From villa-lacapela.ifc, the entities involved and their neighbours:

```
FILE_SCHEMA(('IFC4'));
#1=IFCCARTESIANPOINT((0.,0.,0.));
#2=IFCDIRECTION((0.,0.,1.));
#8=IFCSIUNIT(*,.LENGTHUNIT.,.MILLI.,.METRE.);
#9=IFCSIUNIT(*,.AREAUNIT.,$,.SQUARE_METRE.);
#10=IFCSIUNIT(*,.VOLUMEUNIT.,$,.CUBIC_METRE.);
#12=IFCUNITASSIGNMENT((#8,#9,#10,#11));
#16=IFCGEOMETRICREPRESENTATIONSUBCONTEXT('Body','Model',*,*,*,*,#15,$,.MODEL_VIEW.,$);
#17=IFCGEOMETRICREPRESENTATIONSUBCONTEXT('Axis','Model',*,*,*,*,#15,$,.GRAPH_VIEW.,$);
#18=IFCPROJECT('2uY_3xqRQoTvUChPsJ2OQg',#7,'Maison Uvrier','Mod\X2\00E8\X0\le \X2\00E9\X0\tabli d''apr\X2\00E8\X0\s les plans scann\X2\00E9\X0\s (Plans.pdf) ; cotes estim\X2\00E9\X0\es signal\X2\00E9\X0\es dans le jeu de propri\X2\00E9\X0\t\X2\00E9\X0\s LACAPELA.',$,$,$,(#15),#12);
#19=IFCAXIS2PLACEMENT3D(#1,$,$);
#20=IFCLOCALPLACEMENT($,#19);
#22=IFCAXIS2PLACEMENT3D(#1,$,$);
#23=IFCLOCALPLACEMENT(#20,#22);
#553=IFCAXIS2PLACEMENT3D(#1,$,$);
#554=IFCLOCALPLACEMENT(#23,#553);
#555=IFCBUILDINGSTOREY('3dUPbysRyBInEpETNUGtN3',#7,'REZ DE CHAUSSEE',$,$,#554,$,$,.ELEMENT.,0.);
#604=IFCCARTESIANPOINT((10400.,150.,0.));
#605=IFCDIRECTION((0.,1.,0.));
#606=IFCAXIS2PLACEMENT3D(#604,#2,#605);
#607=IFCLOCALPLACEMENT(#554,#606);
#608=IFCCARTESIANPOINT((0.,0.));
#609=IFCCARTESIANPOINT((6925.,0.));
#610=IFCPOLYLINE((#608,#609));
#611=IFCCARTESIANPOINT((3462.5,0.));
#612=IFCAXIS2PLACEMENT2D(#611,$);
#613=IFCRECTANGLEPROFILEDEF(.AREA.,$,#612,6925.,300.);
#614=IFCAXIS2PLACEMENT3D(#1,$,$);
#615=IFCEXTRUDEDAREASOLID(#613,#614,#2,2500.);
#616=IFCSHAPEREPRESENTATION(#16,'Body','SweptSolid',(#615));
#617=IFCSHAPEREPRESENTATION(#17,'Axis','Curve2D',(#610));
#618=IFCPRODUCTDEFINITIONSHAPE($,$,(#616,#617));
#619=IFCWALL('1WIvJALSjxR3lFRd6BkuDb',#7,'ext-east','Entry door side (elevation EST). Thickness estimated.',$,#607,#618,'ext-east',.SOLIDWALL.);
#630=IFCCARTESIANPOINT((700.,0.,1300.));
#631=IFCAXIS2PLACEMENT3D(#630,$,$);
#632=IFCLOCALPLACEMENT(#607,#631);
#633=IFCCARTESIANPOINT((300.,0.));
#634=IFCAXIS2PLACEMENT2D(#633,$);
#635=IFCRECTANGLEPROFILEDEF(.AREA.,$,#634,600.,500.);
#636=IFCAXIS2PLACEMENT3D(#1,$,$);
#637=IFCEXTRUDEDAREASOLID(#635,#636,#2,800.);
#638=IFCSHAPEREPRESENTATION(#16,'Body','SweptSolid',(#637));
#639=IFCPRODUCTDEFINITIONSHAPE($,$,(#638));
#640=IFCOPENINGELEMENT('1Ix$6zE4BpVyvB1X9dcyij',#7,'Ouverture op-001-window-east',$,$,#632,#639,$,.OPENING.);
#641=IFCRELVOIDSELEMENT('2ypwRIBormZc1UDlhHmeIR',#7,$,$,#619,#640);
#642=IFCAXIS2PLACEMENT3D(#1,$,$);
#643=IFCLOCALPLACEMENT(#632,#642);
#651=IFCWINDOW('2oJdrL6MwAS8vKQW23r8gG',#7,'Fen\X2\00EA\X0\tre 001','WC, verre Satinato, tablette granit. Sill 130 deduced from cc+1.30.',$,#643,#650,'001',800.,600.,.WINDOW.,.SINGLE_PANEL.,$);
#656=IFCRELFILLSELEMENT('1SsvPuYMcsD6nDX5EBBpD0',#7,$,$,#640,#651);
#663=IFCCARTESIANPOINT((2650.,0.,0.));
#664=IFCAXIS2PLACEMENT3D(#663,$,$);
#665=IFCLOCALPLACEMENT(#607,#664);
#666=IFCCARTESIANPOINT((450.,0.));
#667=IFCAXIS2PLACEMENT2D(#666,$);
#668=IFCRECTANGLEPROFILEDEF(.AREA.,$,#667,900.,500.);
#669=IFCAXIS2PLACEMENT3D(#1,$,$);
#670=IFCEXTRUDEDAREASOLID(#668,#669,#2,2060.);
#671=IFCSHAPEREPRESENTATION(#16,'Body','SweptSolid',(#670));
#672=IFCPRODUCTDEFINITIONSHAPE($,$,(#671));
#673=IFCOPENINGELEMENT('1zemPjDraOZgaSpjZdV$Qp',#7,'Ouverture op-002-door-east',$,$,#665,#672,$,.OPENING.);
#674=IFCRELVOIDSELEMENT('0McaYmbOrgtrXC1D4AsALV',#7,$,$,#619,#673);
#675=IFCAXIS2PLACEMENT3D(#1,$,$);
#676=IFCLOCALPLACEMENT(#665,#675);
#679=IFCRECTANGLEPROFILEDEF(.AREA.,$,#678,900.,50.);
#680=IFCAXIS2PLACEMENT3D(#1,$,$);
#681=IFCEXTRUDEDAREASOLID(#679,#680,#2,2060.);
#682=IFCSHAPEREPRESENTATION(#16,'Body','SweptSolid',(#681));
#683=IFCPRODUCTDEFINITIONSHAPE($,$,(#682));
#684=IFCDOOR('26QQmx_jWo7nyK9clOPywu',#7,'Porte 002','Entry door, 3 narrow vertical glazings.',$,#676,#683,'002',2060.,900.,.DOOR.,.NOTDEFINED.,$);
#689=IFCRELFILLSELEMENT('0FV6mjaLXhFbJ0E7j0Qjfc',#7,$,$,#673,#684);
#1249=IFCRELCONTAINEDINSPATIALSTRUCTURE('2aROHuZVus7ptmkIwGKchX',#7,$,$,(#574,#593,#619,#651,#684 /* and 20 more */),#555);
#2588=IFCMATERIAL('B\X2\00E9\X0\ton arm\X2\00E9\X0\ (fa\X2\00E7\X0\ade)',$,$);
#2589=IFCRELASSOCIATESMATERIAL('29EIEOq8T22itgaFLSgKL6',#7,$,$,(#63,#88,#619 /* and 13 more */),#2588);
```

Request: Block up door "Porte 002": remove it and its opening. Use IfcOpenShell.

```python
import ifcopenshell
import ifcopenshell.api.feature
import ifcopenshell.api.root
import ifcopenshell.geom
import ifcopenshell.util.shape

model = ifcopenshell.open("villa-lacapela.ifc")
settings = ifcopenshell.geom.settings()


def volume(element):
    """Net volume in cubic metres, openings subtracted."""
    shape = ifcopenshell.geom.create_shape(settings, element)
    return ifcopenshell.util.shape.get_volume(shape.geometry)


door = model.by_guid("26QQmx_jWo7nyK9clOPywu")
opening = door.FillsVoids[0].RelatingOpeningElement
wall = opening.VoidsElements[0].RelatingBuildingElement
before = volume(wall)

ifcopenshell.api.root.remove_product(model, product=door)
ifcopenshell.api.feature.remove_feature(model, feature=opening)

after = volume(wall)

print(f"wall volume {before:.3f} -> {after:.3f} m3")

model.write("villa-lacapela_rev.ifc")
```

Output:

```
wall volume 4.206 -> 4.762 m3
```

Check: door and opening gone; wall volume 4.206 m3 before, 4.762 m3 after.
